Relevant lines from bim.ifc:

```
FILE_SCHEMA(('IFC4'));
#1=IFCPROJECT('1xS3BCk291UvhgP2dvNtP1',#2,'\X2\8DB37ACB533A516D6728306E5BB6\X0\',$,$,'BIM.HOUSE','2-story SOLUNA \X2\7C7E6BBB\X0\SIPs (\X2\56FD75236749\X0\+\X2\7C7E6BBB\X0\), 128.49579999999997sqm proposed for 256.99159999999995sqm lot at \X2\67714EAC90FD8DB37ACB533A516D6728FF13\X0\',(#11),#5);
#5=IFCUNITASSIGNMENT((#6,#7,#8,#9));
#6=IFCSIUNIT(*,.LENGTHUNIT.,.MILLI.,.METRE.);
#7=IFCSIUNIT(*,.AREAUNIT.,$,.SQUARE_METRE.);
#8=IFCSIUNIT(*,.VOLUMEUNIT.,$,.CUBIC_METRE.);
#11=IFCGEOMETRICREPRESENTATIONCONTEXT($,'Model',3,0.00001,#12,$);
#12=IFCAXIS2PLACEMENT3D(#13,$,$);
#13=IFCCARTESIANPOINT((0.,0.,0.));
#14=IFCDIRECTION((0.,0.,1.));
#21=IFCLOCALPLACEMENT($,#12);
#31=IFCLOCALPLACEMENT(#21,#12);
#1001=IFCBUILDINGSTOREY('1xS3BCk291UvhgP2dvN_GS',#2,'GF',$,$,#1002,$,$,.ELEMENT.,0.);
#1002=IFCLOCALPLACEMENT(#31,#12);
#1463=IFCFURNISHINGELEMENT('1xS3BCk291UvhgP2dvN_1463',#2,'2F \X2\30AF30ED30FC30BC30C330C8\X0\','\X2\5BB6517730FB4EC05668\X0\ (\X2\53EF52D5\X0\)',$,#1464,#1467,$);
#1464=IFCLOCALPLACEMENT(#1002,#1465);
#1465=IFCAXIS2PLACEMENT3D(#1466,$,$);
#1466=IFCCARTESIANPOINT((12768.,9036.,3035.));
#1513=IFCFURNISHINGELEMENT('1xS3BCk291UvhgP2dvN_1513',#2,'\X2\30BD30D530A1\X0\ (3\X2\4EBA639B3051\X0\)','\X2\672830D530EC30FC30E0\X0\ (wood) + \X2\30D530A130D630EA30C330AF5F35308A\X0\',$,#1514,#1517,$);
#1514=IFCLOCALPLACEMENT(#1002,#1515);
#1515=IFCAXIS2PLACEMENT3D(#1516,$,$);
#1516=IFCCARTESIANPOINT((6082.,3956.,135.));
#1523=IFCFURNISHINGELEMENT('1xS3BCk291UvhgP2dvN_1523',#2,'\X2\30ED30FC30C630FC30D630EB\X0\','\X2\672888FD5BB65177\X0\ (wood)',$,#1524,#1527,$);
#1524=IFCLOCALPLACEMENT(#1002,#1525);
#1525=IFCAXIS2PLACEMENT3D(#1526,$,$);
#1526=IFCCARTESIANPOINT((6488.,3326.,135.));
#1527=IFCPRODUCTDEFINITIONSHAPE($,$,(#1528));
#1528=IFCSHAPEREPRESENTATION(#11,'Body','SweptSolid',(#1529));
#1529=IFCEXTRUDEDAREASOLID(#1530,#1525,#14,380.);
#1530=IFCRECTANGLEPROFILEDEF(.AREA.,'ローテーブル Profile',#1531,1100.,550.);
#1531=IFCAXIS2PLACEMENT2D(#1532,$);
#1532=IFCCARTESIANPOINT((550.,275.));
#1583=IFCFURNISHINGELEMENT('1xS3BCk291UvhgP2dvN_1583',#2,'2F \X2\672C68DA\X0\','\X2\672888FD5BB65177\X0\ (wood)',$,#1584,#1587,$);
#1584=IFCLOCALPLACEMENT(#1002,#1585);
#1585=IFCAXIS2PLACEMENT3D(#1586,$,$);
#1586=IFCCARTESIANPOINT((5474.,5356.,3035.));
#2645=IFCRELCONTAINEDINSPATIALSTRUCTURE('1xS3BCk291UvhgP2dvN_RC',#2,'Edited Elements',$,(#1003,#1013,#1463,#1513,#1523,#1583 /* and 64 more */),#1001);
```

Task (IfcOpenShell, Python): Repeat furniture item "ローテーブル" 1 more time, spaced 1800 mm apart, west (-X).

```python
import numpy as np
import ifcopenshell
import ifcopenshell.api.geometry
import ifcopenshell.api.root
import ifcopenshell.util.element
import ifcopenshell.util.placement
import ifcopenshell.util.unit

model = ifcopenshell.open("bim.ifc")
unit_scale = ifcopenshell.util.unit.calculate_unit_scale(model)


def reuse_history(source, copy):
    """copy_class also copies each property set's owner history, people and application; keep the originals."""
    for rel in copy.IsDefinedBy:
        if rel.is_a("IfcRelDefinesByProperties") and (history := rel.RelatingPropertyDefinition.OwnerHistory):
            rel.RelatingPropertyDefinition.OwnerHistory = source.OwnerHistory
            ifcopenshell.util.element.remove_deep2(model, history)


source = model.by_guid("1xS3BCk291UvhgP2dvN_1523")
base = ifcopenshell.util.placement.get_local_placement(source.ObjectPlacement)
step = np.array([-1.0, 0.0, 0.0]) * 1.8 / unit_scale

for i in range(1, 2):
    copy = ifcopenshell.api.root.copy_class(model, product=source)
    copy.Representation = ifcopenshell.util.element.copy_deep(
        model, source.Representation, exclude=["IfcGeometricRepresentationContext", "IfcRepresentationMap"]
    )
    reuse_history(source, copy)
    matrix = base.copy()
    matrix[:3, 3] += i * step
    print("added at", matrix[:3, 3].round(3) + 0.0)
    ifcopenshell.api.geometry.edit_object_placement(model, product=copy, matrix=matrix, is_si=False)

model.write("bim_v2.ifc")
```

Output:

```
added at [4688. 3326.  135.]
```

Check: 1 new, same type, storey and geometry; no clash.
